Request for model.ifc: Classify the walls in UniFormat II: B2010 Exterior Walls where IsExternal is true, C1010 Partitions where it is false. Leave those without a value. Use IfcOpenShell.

First a look at what the model holds.

```python
import ifcopenshell
import ifcopenshell.util.element

model = ifcopenshell.open("model.ifc")
print(model.schema)
print("classifications:", [c.Name for c in model.by_type("IfcClassification")])
values = [ifcopenshell.util.element.get_pset(e, "Pset_WallCommon", "IsExternal") for e in model.by_type("IfcWall")]
for value in (True, False, None):
    print("IsExternal", value, values.count(value))
```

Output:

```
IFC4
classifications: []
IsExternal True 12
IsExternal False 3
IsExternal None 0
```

```python
import ifcopenshell
import ifcopenshell.api.classification
import ifcopenshell.util.element

model = ifcopenshell.open("model.ifc")

system = ifcopenshell.api.classification.add_classification(model, classification="UniFormat II")

walls = model.by_type("IfcWall")
external = {e: ifcopenshell.util.element.get_pset(e, "Pset_WallCommon", "IsExternal") for e in walls}
for flag, code, name in ((True, "B2010", "Exterior Walls"), (False, "C1010", "Partitions")):
    products = [e for e in walls if external[e] is flag]
    ifcopenshell.api.classification.add_reference(
        model, products=products, classification=system, identification=code, name=name
    )
    print(code, len(products))

model.write("model_edited.ifc")
```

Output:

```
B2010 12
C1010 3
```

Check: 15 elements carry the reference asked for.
